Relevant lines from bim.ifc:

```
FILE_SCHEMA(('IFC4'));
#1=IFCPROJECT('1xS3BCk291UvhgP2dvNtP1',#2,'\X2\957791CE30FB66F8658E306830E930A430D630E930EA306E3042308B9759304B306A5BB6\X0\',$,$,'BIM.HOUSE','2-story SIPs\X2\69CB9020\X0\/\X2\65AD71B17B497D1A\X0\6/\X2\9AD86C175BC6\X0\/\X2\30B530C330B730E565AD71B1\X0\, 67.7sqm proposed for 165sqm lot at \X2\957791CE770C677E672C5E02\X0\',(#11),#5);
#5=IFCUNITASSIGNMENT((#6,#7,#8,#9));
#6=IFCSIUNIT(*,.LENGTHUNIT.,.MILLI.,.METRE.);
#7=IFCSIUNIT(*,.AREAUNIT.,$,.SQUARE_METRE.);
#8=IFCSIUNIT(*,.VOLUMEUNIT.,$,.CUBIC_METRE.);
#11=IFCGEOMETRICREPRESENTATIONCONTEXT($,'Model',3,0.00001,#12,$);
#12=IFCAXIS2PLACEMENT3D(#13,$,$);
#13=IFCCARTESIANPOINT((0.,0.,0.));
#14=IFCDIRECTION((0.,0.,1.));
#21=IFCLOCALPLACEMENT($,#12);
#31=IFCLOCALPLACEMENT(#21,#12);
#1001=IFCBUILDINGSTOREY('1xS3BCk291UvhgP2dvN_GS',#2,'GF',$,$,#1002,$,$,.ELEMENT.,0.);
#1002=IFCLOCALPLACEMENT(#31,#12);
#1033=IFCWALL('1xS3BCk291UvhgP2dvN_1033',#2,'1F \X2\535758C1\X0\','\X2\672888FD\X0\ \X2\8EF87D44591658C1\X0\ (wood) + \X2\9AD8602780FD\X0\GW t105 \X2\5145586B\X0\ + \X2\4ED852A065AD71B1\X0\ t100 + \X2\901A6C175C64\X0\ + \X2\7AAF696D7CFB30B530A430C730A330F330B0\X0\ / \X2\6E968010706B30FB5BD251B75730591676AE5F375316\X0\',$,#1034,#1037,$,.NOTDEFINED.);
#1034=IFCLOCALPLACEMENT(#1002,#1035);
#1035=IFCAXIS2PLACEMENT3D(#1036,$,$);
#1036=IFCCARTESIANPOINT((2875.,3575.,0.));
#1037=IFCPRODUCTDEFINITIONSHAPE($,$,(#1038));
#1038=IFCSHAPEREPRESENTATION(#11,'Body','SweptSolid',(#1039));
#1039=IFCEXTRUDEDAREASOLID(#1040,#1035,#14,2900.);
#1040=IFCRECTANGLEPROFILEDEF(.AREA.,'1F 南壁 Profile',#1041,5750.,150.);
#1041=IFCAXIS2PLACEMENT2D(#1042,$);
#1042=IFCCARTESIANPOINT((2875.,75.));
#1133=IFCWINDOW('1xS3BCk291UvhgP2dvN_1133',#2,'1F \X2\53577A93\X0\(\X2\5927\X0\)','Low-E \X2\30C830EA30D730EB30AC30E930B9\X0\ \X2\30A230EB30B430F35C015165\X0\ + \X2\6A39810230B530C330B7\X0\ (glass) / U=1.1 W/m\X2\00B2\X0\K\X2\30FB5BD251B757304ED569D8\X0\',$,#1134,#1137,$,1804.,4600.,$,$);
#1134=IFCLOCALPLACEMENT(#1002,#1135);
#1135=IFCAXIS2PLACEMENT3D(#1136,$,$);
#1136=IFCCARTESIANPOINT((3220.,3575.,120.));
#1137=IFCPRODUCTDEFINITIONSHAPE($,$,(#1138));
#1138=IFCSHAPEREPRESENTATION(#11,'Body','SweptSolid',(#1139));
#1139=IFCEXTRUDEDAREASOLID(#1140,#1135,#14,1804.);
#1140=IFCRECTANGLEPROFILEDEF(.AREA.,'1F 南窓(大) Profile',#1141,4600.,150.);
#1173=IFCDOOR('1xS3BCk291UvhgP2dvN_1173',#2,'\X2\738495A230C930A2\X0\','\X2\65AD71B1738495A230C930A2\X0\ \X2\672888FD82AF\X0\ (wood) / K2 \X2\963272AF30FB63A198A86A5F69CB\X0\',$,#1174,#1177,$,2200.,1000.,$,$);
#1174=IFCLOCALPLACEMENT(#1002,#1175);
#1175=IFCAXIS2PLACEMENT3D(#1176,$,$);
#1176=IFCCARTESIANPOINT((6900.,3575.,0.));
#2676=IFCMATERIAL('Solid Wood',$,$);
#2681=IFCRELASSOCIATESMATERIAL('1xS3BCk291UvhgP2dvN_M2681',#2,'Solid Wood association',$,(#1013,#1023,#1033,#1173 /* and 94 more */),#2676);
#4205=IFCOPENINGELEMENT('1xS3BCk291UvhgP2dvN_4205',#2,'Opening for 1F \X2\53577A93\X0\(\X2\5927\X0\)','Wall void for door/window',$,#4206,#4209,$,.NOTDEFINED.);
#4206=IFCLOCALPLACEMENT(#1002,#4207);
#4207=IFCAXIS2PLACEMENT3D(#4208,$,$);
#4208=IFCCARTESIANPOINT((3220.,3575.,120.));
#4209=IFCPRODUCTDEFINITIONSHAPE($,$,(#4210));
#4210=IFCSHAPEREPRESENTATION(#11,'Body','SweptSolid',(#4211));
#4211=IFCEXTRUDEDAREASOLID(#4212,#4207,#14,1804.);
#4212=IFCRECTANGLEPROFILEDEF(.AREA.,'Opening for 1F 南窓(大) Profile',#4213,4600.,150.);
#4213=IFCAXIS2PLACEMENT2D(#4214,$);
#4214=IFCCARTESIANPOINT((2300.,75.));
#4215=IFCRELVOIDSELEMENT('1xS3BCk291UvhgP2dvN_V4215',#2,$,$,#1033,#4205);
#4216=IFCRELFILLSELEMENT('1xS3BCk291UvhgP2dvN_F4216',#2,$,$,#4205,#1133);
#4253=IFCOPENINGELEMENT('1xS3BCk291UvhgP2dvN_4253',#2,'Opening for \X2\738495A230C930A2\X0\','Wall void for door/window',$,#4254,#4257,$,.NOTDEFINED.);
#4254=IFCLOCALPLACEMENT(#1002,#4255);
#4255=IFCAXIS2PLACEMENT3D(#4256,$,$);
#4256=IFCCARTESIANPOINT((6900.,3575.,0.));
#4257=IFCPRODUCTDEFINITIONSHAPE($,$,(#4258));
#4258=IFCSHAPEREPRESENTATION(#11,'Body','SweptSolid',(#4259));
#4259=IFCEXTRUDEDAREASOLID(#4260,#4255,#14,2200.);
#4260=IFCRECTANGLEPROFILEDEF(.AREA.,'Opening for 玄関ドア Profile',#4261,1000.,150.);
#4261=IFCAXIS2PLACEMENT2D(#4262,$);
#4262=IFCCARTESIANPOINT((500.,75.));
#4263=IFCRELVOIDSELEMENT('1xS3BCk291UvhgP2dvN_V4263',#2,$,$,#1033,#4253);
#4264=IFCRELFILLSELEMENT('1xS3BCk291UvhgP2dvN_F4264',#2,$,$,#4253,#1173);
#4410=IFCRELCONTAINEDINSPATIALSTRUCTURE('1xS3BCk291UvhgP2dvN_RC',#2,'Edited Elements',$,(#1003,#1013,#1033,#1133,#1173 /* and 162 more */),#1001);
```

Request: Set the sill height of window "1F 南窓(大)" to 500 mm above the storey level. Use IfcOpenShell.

```python
import numpy as np
import ifcopenshell
import ifcopenshell.api.geometry
import ifcopenshell.geom
import ifcopenshell.util.element
import ifcopenshell.util.placement
import ifcopenshell.util.shape
import ifcopenshell.util.unit

model = ifcopenshell.open("bim.ifc")
unit_scale = ifcopenshell.util.unit.calculate_unit_scale(model)

window = model.by_id(1133)
opening = window.FillsVoids[0].RelatingOpeningElement
storey = ifcopenshell.util.element.get_container(window, ifc_class="IfcBuildingStorey")
level = ifcopenshell.util.placement.get_local_placement(storey.ObjectPlacement)[2, 3]

# The opening's origin need not be at the sill, so measure its lowest point.
shape = ifcopenshell.geom.create_shape(ifcopenshell.geom.settings(), opening)
bottom = ifcopenshell.util.shape.get_shape_bottom_elevation(shape, shape.geometry) / unit_scale
dz = level + 0.5 / unit_scale - bottom

shift = np.array([0.0, 0.0, dz])
# The window is not placed relative to its opening, so move both.
for product in (opening, window):
    matrix = ifcopenshell.util.placement.get_local_placement(product.ObjectPlacement)
    matrix[:3, 3] += shift
    ifcopenshell.api.geometry.edit_object_placement(model, product=product, matrix=matrix, is_si=False)

print(f"moved by {dz * unit_scale:+.3f} m")

model.write("bim-out.ifc")
```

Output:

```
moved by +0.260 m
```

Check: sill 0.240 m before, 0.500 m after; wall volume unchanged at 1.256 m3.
